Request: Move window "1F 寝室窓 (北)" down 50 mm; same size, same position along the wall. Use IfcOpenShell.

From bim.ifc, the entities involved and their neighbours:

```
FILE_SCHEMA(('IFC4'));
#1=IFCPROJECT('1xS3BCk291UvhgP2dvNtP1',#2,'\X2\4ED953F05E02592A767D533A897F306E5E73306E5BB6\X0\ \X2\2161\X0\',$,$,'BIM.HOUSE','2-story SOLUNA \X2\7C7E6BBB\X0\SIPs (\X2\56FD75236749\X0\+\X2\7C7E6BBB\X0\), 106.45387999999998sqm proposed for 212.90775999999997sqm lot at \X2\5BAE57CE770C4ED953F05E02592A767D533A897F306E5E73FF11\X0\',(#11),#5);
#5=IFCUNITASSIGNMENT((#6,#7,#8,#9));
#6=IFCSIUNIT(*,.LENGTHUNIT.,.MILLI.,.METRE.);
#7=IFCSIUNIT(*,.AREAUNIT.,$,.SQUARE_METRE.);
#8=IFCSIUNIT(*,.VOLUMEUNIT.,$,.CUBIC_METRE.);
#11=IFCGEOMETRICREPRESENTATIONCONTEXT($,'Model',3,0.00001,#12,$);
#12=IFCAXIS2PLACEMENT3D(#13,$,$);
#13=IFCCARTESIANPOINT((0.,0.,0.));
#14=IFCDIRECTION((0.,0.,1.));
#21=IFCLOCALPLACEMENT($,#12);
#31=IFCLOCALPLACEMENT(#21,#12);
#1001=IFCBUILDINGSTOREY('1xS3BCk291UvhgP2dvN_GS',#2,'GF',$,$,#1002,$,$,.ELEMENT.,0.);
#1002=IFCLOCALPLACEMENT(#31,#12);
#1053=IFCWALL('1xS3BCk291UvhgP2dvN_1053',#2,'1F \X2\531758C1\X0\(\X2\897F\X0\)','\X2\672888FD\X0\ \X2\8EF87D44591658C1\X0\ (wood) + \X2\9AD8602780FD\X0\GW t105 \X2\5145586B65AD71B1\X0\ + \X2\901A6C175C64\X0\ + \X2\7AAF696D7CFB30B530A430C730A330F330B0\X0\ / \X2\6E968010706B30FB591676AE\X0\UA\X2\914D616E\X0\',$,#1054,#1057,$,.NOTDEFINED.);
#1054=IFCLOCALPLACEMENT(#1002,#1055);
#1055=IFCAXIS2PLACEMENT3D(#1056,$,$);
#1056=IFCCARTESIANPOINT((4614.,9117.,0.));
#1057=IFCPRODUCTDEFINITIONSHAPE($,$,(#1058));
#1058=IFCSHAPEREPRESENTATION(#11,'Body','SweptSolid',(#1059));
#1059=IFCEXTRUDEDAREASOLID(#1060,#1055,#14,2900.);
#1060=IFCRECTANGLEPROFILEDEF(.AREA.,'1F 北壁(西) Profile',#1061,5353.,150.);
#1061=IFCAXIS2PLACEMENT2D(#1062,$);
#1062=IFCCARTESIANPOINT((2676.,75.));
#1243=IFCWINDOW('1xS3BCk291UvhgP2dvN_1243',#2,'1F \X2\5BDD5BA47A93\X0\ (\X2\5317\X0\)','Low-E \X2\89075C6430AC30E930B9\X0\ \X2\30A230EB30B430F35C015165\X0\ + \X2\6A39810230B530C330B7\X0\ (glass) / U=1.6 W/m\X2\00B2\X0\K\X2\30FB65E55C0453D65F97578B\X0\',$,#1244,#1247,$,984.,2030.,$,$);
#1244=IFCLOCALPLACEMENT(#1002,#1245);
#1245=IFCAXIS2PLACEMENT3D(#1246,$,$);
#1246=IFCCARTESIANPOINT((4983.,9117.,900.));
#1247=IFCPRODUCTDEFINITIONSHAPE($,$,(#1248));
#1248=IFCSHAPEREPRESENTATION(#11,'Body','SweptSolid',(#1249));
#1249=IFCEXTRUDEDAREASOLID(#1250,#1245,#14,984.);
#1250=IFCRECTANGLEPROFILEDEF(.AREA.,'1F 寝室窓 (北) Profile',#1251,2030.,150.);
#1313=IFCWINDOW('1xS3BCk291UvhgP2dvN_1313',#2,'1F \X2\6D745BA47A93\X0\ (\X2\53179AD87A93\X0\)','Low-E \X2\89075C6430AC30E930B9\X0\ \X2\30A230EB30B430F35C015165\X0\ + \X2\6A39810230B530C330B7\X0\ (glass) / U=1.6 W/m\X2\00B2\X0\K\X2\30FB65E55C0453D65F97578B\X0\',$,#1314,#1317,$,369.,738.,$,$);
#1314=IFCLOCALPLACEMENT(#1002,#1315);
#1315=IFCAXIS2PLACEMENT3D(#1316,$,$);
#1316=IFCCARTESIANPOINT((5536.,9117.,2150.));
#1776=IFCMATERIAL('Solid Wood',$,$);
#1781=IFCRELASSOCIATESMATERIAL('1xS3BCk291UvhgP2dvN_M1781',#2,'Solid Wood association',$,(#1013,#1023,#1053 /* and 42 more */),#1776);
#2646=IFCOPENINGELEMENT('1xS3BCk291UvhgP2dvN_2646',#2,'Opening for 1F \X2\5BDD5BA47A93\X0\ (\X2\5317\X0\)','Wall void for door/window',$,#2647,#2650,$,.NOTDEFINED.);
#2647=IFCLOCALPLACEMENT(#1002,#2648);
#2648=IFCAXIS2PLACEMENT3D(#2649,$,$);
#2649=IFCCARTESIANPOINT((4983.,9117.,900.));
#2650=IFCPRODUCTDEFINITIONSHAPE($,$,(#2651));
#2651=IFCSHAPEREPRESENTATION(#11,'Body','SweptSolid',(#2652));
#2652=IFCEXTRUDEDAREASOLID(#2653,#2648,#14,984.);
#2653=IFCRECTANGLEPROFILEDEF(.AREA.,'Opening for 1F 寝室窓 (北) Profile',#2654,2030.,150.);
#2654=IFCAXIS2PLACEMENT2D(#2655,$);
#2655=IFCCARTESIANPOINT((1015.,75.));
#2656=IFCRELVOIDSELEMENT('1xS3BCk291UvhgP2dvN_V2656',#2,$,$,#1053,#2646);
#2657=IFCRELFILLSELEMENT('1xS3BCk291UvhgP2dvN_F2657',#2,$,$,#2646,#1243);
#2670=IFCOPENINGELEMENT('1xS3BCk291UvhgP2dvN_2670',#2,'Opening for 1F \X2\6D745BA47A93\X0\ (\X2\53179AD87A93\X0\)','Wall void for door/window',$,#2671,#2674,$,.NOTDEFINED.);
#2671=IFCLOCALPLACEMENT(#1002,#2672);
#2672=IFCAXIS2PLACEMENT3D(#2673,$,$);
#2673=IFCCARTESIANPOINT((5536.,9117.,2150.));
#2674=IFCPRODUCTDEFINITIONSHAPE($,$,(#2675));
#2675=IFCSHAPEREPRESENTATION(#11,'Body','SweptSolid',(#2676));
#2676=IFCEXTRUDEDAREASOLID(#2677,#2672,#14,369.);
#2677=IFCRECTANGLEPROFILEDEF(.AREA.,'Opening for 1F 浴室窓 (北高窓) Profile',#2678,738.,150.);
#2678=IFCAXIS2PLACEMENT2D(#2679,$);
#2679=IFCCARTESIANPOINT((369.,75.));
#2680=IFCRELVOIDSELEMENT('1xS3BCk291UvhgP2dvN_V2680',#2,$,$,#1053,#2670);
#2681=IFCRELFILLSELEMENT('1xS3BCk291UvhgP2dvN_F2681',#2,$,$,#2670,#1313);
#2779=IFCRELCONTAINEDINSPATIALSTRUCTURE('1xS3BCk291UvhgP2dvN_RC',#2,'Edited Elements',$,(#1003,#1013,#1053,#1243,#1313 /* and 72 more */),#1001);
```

```python
import numpy as np
import ifcopenshell
import ifcopenshell.api.geometry
import ifcopenshell.util.placement
import ifcopenshell.util.unit

model = ifcopenshell.open("bim.ifc")
unit_scale = ifcopenshell.util.unit.calculate_unit_scale(model)

window = model.by_id(1243)
opening = window.FillsVoids[0].RelatingOpeningElement
dz = -50.0

shift = np.array([0.0, 0.0, dz])
# The window is not placed relative to its opening, so move both.
for product in (opening, window):
    matrix = ifcopenshell.util.placement.get_local_placement(product.ObjectPlacement)
    matrix[:3, 3] += shift
    ifcopenshell.api.geometry.edit_object_placement(model, product=product, matrix=matrix, is_si=False)

print(f"moved by {dz * unit_scale:+.3f} m")

model.write("bim_updated.ifc")
```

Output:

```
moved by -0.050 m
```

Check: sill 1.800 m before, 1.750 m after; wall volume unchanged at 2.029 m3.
